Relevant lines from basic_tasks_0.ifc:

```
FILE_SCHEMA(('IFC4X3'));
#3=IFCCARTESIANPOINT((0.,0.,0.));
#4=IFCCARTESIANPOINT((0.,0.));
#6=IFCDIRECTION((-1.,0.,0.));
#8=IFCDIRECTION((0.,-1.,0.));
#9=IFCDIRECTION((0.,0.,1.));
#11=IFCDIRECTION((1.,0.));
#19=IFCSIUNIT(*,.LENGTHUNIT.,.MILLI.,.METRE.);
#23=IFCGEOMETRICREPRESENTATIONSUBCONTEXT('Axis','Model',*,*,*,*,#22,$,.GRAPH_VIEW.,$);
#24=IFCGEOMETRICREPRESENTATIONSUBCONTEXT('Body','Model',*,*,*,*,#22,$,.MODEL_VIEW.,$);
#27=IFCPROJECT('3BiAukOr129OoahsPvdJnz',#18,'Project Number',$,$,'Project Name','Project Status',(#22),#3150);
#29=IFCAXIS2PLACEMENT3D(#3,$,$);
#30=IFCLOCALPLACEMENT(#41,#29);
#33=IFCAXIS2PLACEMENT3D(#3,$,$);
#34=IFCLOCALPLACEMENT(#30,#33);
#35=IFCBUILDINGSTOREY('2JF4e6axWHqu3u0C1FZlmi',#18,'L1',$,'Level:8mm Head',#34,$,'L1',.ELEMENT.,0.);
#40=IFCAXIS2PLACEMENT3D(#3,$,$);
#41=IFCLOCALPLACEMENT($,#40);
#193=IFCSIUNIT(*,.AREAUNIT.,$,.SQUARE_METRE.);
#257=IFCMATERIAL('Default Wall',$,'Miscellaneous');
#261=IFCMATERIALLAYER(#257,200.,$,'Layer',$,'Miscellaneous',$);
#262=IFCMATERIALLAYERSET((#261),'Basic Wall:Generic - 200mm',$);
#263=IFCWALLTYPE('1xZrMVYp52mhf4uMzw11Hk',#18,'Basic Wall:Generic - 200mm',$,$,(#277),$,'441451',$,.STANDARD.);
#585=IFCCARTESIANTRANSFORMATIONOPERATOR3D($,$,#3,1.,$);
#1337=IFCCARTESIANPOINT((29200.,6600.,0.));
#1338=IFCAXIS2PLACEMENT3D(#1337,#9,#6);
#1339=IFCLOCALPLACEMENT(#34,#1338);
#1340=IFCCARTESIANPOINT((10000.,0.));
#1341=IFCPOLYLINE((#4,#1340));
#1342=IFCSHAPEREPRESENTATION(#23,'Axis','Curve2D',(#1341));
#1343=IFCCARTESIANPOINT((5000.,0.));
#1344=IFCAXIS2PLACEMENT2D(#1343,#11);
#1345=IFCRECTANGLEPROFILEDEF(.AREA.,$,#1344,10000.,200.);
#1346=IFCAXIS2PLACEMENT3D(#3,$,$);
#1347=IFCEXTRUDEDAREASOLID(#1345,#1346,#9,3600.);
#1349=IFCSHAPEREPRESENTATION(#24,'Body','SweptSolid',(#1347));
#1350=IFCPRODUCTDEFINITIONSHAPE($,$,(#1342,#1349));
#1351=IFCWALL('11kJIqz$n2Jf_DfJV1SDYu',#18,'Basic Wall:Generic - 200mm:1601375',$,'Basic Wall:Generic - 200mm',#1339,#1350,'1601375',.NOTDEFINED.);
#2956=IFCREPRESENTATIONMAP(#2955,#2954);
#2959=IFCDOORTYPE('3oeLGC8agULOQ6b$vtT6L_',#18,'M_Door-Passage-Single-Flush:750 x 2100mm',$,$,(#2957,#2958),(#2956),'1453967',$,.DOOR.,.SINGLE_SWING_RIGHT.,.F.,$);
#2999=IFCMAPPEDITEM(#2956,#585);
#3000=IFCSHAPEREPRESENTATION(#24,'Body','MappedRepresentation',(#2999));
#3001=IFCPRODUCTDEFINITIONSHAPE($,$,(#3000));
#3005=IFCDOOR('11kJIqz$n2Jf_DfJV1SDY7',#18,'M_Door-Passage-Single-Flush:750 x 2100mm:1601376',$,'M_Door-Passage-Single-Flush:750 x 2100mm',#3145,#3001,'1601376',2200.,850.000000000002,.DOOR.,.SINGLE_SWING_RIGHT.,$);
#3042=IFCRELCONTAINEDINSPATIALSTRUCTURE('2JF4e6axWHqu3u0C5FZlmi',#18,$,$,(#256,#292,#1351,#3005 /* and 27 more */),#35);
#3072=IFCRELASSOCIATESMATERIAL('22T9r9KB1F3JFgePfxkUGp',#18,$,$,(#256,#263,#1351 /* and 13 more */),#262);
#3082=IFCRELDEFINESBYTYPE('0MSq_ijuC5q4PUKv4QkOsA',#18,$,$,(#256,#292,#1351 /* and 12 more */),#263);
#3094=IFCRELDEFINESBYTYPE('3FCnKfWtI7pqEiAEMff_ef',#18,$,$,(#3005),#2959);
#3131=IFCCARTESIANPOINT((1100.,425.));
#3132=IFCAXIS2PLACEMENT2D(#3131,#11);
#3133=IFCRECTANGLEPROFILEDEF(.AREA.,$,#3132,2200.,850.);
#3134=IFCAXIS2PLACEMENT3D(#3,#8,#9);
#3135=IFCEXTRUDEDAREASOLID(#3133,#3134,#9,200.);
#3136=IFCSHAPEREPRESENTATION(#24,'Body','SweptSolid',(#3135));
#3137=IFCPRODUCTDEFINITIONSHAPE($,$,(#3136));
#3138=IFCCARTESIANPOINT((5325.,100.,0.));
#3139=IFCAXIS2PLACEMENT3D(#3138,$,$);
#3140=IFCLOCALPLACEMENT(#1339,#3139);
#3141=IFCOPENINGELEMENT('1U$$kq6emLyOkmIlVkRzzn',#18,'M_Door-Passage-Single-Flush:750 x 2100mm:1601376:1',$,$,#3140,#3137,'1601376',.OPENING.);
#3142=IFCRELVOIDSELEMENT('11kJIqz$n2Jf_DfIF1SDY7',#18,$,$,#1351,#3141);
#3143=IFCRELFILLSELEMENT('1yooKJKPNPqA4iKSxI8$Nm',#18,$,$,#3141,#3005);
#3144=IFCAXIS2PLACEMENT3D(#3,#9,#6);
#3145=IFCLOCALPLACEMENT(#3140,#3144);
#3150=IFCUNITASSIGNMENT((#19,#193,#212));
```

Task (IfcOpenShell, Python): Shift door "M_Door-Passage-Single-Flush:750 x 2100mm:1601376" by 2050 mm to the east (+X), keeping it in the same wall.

```python
import ifcopenshell
import ifcopenshell.api.geometry
import ifcopenshell.util.placement
import ifcopenshell.util.unit

model = ifcopenshell.open("basic_tasks_0.ifc")
unit_scale = ifcopenshell.util.unit.calculate_unit_scale(model)

door = model.by_guid("11kJIqz$n2Jf_DfJV1SDY7")
opening = door.FillsVoids[0].RelatingOpeningElement
wall = opening.VoidsElements[0].RelatingBuildingElement

wall_matrix = ifcopenshell.util.placement.get_local_placement(wall.ObjectPlacement)
shift = wall_matrix[:3, 0] * -2.05 / unit_scale
before = ifcopenshell.util.placement.get_local_placement(door.ObjectPlacement)[:3, 3].copy()

# The door is placed relative to its opening, so it follows when the opening moves.
matrix = ifcopenshell.util.placement.get_local_placement(opening.ObjectPlacement)
matrix[:3, 3] += shift
ifcopenshell.api.geometry.edit_object_placement(
    model, product=opening, matrix=matrix, is_si=False, should_transform_children=True
)

after = ifcopenshell.util.placement.get_local_placement(door.ObjectPlacement)[:3, 3]
print("door moved by", (after - before).round(3) + 0.0)

model.write("basic_tasks_0_rev.ifc")
```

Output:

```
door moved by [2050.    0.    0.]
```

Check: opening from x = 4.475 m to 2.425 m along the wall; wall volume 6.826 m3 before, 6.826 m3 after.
